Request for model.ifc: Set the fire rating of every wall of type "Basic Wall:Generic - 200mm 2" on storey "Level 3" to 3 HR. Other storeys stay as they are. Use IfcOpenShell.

First a look at what the model holds.

```python
import ifcopenshell
import ifcopenshell.util.element

model = ifcopenshell.open("model.ifc")
print(model.schema)
storey = next(s for s in model.by_type("IfcBuildingStorey") if s.Name == "Level 3")
walls = [e for e in ifcopenshell.util.element.get_decomposition(storey) if e.is_a("IfcWall")]
seen = {}
for e in walls:
    element_type = ifcopenshell.util.element.get_type(e)
    key = (element_type.Name if element_type != e and element_type else None, ifcopenshell.util.element.get_pset(e, "Pset_WallCommon", "FireRating"))
    seen[key] = seen.get(key, 0) + 1
for (name, value), count in sorted(seen.items(), key=str):
    print(count, "x", name, "|", value)
```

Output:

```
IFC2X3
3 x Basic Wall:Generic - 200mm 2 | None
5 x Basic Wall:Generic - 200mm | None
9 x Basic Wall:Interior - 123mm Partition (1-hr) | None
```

```python
import ifcopenshell
import ifcopenshell.api.pset
import ifcopenshell.util.element

model = ifcopenshell.open("model.ifc")

storey = next(s for s in model.by_type("IfcBuildingStorey") if s.Name == "Level 3")
walls = [e for e in ifcopenshell.util.element.get_decomposition(storey) if e.is_a("IfcWall")]

count = 0
for e in walls:
    element_type = ifcopenshell.util.element.get_type(e)
    if element_type in (None, e) or element_type.Name != "Basic Wall:Generic - 200mm 2":
        continue
    found = ifcopenshell.util.element.get_pset(e, "Pset_WallCommon", should_inherit=False)
    if found:
        pset = model.by_id(found["id"])
        if len(ifcopenshell.util.element.get_elements_by_pset(pset)) > 1:
            pset = ifcopenshell.api.pset.unshare_pset(model, products=[e], pset=pset)[0]
    else:
        pset = ifcopenshell.api.pset.add_pset(model, product=e, name="Pset_WallCommon")
    ifcopenshell.api.pset.edit_pset(model, pset=pset, properties={"FireRating": "3 HR"})
    count += 1

print(count, "walls updated")

model.write("model_rev.ifc")
```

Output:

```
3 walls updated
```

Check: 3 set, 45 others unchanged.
